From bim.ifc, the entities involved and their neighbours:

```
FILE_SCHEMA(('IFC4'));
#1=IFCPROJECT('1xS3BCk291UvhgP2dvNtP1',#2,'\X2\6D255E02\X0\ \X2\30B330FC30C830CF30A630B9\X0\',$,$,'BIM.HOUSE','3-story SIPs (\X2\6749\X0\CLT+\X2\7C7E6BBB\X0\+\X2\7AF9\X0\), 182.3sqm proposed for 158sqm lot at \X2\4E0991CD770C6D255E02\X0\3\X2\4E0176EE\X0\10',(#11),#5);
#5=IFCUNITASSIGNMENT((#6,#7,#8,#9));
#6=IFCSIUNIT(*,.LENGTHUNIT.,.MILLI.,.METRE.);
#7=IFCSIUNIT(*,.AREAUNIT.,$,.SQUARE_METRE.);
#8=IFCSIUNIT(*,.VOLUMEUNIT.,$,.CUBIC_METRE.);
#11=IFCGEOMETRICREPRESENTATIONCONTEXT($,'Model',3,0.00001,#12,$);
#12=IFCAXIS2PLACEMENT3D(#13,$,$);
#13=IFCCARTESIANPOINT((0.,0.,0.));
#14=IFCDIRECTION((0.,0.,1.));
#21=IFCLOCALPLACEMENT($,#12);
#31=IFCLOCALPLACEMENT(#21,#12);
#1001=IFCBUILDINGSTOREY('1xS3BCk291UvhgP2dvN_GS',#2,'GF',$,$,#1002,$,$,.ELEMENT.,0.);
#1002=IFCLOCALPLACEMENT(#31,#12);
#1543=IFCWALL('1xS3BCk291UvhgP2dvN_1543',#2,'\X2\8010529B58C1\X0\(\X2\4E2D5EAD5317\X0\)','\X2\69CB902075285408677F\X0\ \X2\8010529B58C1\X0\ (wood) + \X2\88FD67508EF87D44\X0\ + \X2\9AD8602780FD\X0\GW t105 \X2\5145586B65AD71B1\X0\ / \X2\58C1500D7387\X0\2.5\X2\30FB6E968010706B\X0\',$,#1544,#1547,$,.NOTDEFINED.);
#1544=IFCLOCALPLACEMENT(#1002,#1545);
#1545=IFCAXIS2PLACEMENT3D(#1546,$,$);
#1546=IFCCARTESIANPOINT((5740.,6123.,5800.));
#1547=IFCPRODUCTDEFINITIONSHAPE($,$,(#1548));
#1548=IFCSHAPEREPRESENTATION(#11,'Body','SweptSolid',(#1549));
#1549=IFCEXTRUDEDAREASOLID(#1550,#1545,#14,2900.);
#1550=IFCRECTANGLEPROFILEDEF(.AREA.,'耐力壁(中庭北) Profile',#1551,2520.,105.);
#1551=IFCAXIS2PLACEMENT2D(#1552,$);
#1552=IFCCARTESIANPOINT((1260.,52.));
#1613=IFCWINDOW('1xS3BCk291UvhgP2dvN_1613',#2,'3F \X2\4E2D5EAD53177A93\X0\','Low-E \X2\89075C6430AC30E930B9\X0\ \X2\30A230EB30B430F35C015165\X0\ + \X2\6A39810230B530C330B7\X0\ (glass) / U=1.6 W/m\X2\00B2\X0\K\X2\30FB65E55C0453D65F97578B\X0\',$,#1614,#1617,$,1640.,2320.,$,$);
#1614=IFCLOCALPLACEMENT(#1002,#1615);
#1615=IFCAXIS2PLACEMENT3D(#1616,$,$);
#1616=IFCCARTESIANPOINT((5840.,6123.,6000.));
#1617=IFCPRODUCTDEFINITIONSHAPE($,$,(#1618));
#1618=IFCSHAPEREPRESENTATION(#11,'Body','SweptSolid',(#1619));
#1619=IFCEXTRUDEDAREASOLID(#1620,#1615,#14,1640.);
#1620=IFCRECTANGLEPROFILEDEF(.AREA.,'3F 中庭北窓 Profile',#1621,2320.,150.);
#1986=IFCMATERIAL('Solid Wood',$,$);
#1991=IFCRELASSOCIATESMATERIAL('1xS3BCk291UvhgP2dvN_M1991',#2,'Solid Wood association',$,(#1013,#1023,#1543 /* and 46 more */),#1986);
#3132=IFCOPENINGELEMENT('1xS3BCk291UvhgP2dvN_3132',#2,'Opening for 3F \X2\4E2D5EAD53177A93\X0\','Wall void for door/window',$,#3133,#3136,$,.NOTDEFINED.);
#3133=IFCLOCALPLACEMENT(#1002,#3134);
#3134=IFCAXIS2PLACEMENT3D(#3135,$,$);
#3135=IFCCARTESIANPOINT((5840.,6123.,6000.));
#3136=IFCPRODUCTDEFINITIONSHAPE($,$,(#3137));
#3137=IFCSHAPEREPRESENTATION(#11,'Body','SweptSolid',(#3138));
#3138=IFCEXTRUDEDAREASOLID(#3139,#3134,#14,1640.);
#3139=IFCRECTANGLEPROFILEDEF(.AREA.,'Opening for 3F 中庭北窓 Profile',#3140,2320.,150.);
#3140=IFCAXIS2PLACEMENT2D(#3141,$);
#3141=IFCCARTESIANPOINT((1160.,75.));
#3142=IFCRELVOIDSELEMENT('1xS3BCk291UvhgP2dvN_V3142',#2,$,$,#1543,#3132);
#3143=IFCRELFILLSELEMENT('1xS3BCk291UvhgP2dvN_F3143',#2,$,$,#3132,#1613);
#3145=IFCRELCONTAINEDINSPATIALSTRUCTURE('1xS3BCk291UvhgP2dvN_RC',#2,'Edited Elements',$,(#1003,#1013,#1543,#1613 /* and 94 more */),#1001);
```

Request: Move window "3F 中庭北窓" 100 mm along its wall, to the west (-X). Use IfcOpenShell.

```python
import ifcopenshell
import ifcopenshell.api.geometry
import ifcopenshell.util.placement

model = ifcopenshell.open("bim.ifc")

window = model.by_id(1613)
opening = window.FillsVoids[0].RelatingOpeningElement
wall = opening.VoidsElements[0].RelatingBuildingElement

wall_matrix = ifcopenshell.util.placement.get_local_placement(wall.ObjectPlacement)
shift = wall_matrix[:3, 0] * -100.0
before = ifcopenshell.util.placement.get_local_placement(window.ObjectPlacement)[:3, 3].copy()

# The window is not placed relative to its opening, so move both.
for product in (opening, window):
    matrix = ifcopenshell.util.placement.get_local_placement(product.ObjectPlacement)
    matrix[:3, 3] += shift
    ifcopenshell.api.geometry.edit_object_placement(model, product=product, matrix=matrix, is_si=False)

after = ifcopenshell.util.placement.get_local_placement(window.ObjectPlacement)[:3, 3]
print("window moved by", (after - before).round(3) + 0.0)

model.write("bim_rev.ifc")
```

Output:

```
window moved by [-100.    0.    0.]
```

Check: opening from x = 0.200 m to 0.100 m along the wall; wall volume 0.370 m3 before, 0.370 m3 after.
